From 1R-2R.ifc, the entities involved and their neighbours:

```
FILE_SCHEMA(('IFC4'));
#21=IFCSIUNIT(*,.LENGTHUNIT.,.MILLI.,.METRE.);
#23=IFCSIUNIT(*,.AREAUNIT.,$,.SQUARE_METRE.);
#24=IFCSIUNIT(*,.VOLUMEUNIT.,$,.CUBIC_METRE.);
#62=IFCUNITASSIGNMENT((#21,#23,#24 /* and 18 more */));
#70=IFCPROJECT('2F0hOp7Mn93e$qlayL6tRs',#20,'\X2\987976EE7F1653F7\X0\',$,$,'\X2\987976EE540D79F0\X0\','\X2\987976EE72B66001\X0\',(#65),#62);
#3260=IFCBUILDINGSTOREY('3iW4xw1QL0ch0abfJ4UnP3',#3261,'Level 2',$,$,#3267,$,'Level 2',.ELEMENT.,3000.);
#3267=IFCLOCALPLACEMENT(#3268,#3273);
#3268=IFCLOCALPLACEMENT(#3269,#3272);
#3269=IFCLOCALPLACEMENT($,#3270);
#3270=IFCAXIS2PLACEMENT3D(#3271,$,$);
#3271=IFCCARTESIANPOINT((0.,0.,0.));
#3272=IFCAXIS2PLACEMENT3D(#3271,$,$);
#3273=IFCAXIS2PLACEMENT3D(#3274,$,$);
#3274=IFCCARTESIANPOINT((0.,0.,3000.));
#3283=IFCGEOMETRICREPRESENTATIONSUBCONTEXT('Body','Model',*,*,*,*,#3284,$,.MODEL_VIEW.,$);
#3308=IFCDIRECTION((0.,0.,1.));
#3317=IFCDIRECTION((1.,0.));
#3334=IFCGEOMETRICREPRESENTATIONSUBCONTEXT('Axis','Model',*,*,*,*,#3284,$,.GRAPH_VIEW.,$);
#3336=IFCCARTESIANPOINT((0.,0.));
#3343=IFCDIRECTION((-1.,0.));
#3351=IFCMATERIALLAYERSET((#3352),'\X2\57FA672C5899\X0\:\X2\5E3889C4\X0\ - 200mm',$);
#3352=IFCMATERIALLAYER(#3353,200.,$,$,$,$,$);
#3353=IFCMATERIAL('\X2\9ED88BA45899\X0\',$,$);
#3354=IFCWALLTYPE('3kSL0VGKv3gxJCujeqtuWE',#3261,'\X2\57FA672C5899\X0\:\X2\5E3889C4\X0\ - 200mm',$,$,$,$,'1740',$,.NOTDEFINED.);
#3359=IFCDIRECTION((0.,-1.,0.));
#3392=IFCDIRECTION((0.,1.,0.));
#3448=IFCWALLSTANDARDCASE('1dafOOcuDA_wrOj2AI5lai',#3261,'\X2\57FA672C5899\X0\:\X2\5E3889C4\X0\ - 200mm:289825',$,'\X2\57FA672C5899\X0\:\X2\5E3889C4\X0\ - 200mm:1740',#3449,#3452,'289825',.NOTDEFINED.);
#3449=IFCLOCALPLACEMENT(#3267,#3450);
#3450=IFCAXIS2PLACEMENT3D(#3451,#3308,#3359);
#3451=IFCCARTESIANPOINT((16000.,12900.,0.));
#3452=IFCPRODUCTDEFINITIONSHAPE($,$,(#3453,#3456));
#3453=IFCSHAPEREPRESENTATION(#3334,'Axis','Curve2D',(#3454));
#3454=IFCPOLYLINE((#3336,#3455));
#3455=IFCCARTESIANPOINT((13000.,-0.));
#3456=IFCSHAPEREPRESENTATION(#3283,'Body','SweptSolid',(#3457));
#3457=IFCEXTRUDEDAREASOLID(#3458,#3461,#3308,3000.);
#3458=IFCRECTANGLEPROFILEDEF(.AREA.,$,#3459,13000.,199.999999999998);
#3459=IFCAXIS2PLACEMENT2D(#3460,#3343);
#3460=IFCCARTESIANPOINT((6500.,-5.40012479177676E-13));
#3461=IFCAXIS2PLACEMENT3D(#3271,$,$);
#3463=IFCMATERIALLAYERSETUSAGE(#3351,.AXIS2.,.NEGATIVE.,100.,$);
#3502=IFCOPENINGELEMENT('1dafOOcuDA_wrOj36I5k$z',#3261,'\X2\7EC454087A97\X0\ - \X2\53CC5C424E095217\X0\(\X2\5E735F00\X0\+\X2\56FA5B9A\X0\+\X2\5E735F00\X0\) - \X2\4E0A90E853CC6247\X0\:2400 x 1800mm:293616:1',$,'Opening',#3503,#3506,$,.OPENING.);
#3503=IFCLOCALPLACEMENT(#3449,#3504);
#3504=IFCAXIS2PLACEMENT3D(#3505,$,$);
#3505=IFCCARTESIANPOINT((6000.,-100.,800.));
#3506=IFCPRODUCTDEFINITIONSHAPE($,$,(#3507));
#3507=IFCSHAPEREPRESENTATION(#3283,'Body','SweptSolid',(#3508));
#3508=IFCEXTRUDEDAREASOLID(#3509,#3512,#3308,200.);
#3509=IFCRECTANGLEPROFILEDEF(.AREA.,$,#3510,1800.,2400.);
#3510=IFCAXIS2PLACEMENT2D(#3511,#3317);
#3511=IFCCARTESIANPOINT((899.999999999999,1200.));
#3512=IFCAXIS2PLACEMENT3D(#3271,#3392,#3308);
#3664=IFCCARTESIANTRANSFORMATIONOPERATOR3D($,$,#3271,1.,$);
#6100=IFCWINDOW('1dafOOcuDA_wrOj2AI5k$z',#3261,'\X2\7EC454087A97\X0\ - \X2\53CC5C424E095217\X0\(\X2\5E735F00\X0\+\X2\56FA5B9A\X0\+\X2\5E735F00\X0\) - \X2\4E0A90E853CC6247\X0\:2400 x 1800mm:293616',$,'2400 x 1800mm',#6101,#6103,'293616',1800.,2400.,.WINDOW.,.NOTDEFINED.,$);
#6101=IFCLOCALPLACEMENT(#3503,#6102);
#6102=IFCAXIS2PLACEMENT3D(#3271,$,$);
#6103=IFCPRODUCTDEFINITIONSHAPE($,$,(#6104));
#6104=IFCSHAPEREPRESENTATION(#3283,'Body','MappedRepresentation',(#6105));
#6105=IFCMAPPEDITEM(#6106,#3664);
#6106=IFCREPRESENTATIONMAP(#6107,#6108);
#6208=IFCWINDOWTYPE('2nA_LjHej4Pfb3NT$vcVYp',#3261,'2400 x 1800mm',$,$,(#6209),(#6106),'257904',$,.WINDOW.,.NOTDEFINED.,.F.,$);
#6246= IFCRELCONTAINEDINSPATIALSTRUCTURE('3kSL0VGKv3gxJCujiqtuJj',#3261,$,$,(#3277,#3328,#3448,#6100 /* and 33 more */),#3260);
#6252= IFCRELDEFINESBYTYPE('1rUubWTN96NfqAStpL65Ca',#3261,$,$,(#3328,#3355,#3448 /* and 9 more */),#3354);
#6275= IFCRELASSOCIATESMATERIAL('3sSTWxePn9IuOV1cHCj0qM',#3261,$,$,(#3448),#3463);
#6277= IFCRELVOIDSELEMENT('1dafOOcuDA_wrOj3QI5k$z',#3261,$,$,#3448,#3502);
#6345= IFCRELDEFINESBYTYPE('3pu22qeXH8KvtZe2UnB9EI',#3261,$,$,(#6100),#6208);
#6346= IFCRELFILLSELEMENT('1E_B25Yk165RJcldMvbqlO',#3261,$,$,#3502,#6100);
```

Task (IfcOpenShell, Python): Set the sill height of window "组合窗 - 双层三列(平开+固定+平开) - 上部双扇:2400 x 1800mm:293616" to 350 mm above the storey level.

```python
import numpy as np
import ifcopenshell
import ifcopenshell.api.geometry
import ifcopenshell.geom
import ifcopenshell.util.element
import ifcopenshell.util.placement
import ifcopenshell.util.shape
import ifcopenshell.util.unit

model = ifcopenshell.open("1R-2R.ifc")
unit_scale = ifcopenshell.util.unit.calculate_unit_scale(model)

window = model.by_guid("1dafOOcuDA_wrOj2AI5k$z")
opening = window.FillsVoids[0].RelatingOpeningElement
storey = ifcopenshell.util.element.get_container(window, ifc_class="IfcBuildingStorey")
level = ifcopenshell.util.placement.get_local_placement(storey.ObjectPlacement)[2, 3]

# The opening's origin need not be at the sill, so measure its lowest point.
shape = ifcopenshell.geom.create_shape(ifcopenshell.geom.settings(), opening)
bottom = ifcopenshell.util.shape.get_shape_bottom_elevation(shape, shape.geometry) / unit_scale
dz = level + 0.35 / unit_scale - bottom

shift = np.array([0.0, 0.0, dz])
# The window is placed relative to its opening, so it follows when the opening moves.
matrix = ifcopenshell.util.placement.get_local_placement(opening.ObjectPlacement)
matrix[:3, 3] += shift
ifcopenshell.api.geometry.edit_object_placement(
    model, product=opening, matrix=matrix, is_si=False, should_transform_children=True
)

print(f"moved by {dz * unit_scale:+.3f} m")

model.write("1R-2R_rev.ifc")
```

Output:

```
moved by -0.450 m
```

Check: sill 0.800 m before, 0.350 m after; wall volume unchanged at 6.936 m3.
